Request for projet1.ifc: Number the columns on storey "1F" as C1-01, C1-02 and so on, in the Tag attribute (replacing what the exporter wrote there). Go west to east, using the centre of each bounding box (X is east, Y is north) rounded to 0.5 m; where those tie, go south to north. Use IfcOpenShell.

First a look at what the model holds.

```python
import ifcopenshell
import ifcopenshell.util.element
import ifcopenshell.util.placement

model = ifcopenshell.open("projet1.ifc")
print(model.schema)
storey = next(s for s in model.by_type("IfcBuildingStorey") if s.Name == "1F")
columns = [e for e in ifcopenshell.util.element.get_decomposition(storey) if e.is_a("IfcColumn")]
for e in sorted(columns, key=lambda e: e.id()):
    origin = ifcopenshell.util.placement.get_local_placement(e.ObjectPlacement)[:3, 3]
    print(e.id(), e.Tag, e.Name, origin.round(2) + 0.0, sep=" | ")
```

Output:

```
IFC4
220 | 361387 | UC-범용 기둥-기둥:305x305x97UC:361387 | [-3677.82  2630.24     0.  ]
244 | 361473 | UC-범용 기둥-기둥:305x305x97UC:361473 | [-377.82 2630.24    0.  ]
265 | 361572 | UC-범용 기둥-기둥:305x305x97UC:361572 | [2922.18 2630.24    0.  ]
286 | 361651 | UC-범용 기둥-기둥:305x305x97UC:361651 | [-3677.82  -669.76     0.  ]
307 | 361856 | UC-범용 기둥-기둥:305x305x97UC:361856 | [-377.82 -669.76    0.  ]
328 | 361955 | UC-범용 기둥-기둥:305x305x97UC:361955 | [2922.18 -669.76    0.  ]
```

```python
import ifcopenshell
import ifcopenshell.geom
import ifcopenshell.util.element
import ifcopenshell.util.shape

model = ifcopenshell.open("projet1.ifc")
settings = ifcopenshell.geom.settings()
settings.set("use-world-coords", True)


def centre(element):
    shape = ifcopenshell.geom.create_shape(settings, element)
    return ifcopenshell.util.shape.get_bbox_centroid(shape.geometry)


storey = next(s for s in model.by_type("IfcBuildingStorey") if s.Name == "1F")
columns = [e for e in ifcopenshell.util.element.get_decomposition(storey) if e.is_a("IfcColumn")]

# Insertion points can sit at a corner or the storey origin, so sort by the geometry (in metres).
centres = {e: centre(e) for e in columns}
columns.sort(key=lambda e: (round(centres[e][0] / 0.5), centres[e][1]))

for i, e in enumerate(columns, start=1):
    number = f"C1-{i:02d}"
    e.Tag = number
    print(e.id(), number)

model.write("projet1_v2.ifc")
```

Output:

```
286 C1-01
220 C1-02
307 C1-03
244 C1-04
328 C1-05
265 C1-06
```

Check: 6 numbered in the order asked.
